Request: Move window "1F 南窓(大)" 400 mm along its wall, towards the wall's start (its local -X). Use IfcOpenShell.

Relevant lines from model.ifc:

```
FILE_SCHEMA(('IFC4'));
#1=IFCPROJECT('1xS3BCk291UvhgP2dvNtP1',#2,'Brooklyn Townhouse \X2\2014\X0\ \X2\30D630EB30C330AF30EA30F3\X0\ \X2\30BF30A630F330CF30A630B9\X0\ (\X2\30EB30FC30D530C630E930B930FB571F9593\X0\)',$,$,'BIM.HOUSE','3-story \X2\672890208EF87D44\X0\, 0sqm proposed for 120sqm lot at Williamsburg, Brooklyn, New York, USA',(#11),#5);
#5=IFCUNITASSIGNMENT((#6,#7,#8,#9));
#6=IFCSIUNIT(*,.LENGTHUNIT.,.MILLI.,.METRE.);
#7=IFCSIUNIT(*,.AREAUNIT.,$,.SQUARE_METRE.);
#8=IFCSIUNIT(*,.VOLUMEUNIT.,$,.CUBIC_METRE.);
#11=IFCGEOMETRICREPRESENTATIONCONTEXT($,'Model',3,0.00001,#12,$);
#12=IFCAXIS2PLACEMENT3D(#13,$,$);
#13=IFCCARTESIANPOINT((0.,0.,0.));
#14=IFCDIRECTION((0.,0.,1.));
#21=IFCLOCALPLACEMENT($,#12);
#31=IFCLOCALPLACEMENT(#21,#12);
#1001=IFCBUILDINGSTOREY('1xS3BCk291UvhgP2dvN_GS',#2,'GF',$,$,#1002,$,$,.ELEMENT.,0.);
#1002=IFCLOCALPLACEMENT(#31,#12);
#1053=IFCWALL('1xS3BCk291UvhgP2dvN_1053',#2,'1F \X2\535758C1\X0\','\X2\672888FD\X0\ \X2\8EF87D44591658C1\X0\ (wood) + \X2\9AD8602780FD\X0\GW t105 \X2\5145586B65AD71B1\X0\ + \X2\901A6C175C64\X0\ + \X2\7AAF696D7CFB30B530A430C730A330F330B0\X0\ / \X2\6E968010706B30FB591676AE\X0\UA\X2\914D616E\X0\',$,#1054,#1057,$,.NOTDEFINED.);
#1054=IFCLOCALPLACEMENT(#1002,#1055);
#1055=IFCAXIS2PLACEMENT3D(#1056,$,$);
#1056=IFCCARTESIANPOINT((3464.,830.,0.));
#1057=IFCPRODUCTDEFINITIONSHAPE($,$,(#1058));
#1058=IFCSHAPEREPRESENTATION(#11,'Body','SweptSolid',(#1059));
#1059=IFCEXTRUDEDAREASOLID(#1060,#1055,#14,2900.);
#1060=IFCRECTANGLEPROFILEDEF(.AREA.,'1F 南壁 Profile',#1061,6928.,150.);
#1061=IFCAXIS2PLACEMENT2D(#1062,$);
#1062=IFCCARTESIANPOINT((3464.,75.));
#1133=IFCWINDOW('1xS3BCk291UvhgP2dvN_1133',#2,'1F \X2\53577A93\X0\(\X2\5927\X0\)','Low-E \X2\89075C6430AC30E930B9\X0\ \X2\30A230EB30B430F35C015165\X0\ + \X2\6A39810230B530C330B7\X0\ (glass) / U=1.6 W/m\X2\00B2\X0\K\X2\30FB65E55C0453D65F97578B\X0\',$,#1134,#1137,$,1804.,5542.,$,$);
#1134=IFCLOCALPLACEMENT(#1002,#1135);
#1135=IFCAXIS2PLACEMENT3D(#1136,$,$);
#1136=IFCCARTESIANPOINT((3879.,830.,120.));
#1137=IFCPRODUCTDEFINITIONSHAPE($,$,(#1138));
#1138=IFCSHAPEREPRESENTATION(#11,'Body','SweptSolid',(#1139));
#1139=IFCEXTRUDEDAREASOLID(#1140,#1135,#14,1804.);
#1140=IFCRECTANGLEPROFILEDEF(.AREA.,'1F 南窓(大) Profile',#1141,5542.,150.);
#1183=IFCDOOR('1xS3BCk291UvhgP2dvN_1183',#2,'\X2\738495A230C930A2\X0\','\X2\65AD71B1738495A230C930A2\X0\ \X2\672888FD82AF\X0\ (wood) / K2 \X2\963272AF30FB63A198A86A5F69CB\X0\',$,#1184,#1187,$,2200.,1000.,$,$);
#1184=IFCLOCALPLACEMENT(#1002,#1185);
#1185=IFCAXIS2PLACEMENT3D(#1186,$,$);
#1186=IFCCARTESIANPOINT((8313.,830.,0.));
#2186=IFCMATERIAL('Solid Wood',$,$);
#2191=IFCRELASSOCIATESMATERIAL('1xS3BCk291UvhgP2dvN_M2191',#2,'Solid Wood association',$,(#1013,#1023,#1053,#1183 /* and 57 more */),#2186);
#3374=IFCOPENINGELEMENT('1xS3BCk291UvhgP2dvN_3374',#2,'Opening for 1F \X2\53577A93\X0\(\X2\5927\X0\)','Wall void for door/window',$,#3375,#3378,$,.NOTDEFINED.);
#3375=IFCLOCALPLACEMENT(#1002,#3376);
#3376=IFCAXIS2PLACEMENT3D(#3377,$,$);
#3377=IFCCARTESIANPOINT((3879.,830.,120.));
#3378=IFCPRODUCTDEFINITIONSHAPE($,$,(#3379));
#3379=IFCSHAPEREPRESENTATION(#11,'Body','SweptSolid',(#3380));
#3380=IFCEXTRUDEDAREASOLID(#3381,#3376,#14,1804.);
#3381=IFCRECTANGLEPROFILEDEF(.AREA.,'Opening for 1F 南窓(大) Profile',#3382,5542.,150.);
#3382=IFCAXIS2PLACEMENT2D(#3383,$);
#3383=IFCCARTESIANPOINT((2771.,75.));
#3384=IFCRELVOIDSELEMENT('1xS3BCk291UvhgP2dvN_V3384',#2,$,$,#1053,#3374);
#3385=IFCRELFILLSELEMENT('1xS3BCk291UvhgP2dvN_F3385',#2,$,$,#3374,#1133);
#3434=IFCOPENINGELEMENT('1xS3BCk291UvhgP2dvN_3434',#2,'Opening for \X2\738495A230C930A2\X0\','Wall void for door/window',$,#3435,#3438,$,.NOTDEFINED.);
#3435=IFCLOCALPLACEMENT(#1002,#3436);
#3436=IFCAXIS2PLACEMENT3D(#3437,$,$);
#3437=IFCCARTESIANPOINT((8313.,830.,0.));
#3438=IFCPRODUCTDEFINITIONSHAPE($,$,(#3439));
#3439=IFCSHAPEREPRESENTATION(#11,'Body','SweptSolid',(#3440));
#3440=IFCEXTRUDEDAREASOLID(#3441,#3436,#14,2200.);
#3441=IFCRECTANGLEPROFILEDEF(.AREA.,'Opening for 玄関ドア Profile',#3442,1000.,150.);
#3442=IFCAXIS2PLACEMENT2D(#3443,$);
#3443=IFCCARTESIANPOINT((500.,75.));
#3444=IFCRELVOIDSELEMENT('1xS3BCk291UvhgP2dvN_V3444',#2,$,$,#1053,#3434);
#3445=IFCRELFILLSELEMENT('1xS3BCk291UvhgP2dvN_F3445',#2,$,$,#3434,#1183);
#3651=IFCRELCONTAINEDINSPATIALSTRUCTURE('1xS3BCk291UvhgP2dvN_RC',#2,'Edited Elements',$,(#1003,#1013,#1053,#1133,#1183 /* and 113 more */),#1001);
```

```python
import ifcopenshell
import ifcopenshell.api.geometry
import ifcopenshell.util.placement

model = ifcopenshell.open("model.ifc")

window = model.by_guid("1xS3BCk291UvhgP2dvN_1133")
opening = window.FillsVoids[0].RelatingOpeningElement
wall = opening.VoidsElements[0].RelatingBuildingElement

wall_matrix = ifcopenshell.util.placement.get_local_placement(wall.ObjectPlacement)
shift = wall_matrix[:3, 0] * -400.0
before = ifcopenshell.util.placement.get_local_placement(window.ObjectPlacement)[:3, 3].copy()

# The window is not placed relative to its opening, so move both.
for product in (opening, window):
    matrix = ifcopenshell.util.placement.get_local_placement(product.ObjectPlacement)
    matrix[:3, 3] += shift
    ifcopenshell.api.geometry.edit_object_placement(model, product=product, matrix=matrix, is_si=False)

after = ifcopenshell.util.placement.get_local_placement(window.ObjectPlacement)[:3, 3]
print("window moved by", (after - before).round(3) + 0.0)

model.write("model_edited.ifc")
```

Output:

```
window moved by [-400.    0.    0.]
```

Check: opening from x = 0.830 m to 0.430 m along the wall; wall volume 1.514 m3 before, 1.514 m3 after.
